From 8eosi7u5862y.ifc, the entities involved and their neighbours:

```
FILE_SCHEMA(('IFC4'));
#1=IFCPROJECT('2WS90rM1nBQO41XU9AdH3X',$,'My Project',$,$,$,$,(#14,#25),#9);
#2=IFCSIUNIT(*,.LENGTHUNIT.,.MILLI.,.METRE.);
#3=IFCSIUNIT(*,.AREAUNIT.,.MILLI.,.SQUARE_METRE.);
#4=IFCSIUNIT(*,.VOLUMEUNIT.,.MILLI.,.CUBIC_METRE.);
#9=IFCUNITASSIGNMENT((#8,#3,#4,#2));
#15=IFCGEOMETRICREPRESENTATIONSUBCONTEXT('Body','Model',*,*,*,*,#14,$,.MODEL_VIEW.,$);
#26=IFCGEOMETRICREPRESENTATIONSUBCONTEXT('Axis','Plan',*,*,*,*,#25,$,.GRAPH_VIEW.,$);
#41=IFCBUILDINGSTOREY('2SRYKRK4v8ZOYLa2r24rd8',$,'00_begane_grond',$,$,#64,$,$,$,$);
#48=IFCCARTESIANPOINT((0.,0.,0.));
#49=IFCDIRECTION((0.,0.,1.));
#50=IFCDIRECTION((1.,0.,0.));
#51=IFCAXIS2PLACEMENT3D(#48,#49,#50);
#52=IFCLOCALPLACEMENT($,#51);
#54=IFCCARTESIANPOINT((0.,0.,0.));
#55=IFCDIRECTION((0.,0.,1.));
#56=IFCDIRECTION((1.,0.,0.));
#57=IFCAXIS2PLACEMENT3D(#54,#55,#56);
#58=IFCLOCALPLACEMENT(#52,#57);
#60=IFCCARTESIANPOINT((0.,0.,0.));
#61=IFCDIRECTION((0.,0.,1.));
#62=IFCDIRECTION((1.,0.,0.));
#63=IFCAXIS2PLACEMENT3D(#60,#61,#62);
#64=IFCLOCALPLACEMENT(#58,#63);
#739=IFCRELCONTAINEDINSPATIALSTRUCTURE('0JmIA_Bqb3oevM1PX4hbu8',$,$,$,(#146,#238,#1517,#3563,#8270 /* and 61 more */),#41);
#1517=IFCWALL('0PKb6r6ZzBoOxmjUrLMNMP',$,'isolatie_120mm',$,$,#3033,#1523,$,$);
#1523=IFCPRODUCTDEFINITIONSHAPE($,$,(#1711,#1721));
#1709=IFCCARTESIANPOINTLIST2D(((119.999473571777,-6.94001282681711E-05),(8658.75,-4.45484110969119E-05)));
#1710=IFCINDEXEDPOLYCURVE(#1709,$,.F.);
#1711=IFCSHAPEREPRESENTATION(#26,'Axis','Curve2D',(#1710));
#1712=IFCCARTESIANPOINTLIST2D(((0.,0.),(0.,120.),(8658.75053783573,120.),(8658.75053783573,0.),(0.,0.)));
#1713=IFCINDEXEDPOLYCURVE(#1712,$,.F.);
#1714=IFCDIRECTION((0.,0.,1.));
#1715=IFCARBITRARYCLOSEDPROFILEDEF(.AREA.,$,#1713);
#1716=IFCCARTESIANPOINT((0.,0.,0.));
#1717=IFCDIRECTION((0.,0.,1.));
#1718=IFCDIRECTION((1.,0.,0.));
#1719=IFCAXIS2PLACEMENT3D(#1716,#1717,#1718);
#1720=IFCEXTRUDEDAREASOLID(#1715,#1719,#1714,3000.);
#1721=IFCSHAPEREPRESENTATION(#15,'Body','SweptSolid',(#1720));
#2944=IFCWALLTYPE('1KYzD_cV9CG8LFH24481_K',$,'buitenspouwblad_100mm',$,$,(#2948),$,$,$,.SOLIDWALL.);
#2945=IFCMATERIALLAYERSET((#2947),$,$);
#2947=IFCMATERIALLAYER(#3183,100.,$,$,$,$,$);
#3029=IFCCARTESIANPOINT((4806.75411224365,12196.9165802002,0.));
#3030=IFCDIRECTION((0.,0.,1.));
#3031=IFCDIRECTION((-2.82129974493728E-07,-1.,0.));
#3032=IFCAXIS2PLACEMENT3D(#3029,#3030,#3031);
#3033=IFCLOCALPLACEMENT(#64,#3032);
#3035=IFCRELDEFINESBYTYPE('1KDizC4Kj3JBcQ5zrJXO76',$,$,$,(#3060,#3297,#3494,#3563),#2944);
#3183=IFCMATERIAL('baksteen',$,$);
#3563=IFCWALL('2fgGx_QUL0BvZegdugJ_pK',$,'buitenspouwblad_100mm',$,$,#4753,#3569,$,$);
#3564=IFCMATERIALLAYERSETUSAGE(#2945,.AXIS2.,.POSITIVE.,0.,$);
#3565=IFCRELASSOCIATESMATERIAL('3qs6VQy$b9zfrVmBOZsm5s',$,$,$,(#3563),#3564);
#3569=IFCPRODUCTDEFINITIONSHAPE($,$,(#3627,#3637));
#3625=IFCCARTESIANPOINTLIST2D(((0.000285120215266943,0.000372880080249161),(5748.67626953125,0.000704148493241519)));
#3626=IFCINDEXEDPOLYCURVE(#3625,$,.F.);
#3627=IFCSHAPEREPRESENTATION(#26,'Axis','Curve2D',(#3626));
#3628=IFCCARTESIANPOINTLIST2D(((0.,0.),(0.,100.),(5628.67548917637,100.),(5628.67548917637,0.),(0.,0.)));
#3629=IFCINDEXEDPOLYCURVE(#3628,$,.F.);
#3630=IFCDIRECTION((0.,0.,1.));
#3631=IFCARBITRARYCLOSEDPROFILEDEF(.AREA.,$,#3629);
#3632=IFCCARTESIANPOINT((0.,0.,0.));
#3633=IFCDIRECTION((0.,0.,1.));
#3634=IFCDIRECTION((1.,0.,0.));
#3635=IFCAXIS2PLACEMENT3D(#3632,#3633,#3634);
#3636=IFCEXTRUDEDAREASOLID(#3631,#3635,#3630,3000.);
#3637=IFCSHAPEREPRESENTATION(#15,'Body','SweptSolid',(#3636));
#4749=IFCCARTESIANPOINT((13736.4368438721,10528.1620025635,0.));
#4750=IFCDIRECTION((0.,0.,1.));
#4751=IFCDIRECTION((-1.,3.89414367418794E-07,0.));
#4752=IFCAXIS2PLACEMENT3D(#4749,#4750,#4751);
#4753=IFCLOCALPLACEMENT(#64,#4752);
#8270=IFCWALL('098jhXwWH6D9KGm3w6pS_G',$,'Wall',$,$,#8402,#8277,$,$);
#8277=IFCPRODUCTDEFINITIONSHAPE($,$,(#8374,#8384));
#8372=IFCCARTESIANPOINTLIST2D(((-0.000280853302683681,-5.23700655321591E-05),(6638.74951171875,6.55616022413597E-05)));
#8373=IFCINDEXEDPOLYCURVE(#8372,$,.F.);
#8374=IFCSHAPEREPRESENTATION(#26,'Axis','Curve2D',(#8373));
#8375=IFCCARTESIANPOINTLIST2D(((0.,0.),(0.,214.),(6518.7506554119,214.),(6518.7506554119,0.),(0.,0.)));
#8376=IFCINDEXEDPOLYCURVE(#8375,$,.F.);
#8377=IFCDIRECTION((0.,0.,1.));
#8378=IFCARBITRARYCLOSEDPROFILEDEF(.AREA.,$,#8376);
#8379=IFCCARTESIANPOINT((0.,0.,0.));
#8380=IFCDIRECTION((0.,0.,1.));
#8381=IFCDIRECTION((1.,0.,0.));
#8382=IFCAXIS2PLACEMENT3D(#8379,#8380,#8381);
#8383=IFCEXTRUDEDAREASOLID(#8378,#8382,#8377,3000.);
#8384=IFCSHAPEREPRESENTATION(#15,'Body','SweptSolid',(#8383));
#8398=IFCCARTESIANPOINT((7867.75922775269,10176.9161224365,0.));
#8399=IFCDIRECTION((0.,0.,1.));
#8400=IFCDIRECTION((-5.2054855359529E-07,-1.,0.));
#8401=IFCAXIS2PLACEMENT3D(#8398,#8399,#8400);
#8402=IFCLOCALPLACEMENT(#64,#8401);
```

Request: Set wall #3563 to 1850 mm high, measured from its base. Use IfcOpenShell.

```python
import ifcopenshell
import ifcopenshell.geom
import ifcopenshell.util.representation
import ifcopenshell.util.shape
import ifcopenshell.util.unit

model = ifcopenshell.open("8eosi7u5862y.ifc")
unit_scale = ifcopenshell.util.unit.calculate_unit_scale(model)
settings = ifcopenshell.geom.settings()


def volume(element):
    """Net volume in cubic metres, openings subtracted."""
    shape = ifcopenshell.geom.create_shape(settings, element)
    return ifcopenshell.util.shape.get_volume(shape.geometry)


wall = model.by_guid("2fgGx_QUL0BvZegdugJ_pK")
before = volume(wall)

body = ifcopenshell.util.representation.get_representation(wall, "Model", "Body")
solid = body.Items[0]
old_height = solid.Depth
solid.Depth = 1.85 / unit_scale
after = volume(wall)

print(f"height {old_height:g} -> {solid.Depth:g}, volume {before:.3f} -> {after:.3f} m3")

model.write("8eosi7u5862y-out.ifc")
```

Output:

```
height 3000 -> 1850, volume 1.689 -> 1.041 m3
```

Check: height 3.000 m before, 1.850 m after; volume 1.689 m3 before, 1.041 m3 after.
